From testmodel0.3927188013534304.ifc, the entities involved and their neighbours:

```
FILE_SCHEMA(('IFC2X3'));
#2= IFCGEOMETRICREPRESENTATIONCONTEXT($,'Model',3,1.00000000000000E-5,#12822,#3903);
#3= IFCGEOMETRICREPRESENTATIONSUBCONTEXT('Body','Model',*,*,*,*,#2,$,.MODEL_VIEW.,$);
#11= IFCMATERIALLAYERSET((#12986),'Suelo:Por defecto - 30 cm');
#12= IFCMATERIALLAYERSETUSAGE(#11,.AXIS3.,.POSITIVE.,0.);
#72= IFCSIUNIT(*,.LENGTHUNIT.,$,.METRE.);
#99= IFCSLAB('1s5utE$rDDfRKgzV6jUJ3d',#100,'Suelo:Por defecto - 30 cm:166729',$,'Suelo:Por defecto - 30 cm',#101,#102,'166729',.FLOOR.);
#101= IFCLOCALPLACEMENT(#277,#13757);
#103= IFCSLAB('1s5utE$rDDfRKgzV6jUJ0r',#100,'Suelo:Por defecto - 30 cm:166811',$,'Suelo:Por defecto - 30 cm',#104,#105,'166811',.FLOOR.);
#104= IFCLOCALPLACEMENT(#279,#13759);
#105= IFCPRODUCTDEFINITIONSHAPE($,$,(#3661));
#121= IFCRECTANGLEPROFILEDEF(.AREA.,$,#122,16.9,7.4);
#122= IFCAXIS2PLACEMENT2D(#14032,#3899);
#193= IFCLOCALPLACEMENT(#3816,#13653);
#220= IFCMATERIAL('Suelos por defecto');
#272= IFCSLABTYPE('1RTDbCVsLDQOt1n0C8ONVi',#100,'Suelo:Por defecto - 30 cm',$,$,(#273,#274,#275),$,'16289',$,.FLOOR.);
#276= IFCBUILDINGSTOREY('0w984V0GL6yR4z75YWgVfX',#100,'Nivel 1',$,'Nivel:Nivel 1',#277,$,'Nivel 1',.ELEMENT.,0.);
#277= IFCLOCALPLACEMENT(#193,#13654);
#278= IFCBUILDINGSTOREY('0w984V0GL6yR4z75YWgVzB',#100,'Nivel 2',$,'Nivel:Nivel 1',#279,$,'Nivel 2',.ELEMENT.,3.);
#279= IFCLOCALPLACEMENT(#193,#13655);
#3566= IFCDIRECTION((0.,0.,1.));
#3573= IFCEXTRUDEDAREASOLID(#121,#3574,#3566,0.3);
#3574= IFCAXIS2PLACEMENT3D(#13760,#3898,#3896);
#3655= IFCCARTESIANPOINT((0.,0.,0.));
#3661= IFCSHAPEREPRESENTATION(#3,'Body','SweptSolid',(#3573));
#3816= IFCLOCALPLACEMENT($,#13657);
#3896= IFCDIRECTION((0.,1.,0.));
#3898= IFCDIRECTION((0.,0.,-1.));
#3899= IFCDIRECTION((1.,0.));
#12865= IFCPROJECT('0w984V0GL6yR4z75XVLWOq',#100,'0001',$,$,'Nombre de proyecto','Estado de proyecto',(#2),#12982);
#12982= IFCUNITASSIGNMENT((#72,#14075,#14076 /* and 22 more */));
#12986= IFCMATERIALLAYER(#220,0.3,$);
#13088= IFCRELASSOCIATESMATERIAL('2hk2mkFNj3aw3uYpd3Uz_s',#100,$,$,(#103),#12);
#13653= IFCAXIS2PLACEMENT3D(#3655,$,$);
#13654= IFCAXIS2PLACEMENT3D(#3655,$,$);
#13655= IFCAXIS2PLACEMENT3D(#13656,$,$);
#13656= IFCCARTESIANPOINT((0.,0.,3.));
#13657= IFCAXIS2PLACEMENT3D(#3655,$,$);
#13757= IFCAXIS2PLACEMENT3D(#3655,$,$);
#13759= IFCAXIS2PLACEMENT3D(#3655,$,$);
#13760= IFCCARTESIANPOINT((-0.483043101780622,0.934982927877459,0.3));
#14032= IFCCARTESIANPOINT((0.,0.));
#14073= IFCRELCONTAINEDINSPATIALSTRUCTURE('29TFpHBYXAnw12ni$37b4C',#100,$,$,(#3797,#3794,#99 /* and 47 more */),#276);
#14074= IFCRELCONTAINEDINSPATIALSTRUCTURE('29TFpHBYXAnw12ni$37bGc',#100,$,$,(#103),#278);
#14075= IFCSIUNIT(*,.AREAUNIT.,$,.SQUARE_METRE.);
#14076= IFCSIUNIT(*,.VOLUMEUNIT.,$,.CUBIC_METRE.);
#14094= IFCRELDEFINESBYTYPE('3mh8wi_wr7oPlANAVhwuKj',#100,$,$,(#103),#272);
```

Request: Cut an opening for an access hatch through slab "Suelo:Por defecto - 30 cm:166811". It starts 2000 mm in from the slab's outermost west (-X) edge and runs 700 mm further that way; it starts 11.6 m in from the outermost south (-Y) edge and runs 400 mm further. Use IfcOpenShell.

```python
import numpy as np
import ifcopenshell
import ifcopenshell.api.feature
import ifcopenshell.api.geometry
import ifcopenshell.api.root
import ifcopenshell.geom
import ifcopenshell.util.placement
import ifcopenshell.util.representation
import ifcopenshell.util.shape
import ifcopenshell.util.unit

model = ifcopenshell.open("testmodel0.3927188013534304.ifc")
unit_scale = ifcopenshell.util.unit.calculate_unit_scale(model)
settings = ifcopenshell.geom.settings()


def volume(element):
    """Net volume in cubic metres, openings subtracted."""
    shape = ifcopenshell.geom.create_shape(settings, element)
    return ifcopenshell.util.shape.get_volume(shape.geometry)


slab = model.by_id(103)
before = volume(slab)

# Extent in the slab's own axes, in metres. The edges named are its -X and -Y sides.
slab_shape = ifcopenshell.geom.create_shape(settings, slab)
vertices = ifcopenshell.util.shape.get_vertices(slab_shape.geometry)
x_min, y_min, bottom = vertices.min(axis=0)
top = vertices[:, 2].max()

opening = ifcopenshell.api.root.create_entity(model, ifc_class="IfcOpeningElement", name="Access hatch opening")
context = ifcopenshell.util.representation.get_context(model, "Model", "Body", "MODEL_VIEW")
width, depth = 0.7, 0.4
outline = [(0.0, 0.0), (width, 0.0), (width, depth), (0.0, depth), (0.0, 0.0)]
# Overshoot both faces by 50 mm so the cut is clean.
shape = ifcopenshell.api.geometry.add_slab_representation(
    model, context=context, depth=top - bottom + 0.1, polyline=outline
)
ifcopenshell.api.geometry.assign_representation(model, product=opening, representation=shape)

matrix = ifcopenshell.util.placement.get_local_placement(slab.ObjectPlacement)
matrix[:, 3] = matrix @ np.append(np.array([x_min + 2, y_min + 11.6, bottom - 0.05]) / unit_scale, 1.0)
ifcopenshell.api.geometry.edit_object_placement(model, product=opening, matrix=matrix, is_si=False)
ifcopenshell.api.feature.add_feature(model, feature=opening, element=slab)

after = volume(slab)

print(f"slab volume {before:.3f} -> {after:.3f} m3")

model.write("testmodel0.3927188013534304_updated.ifc")
```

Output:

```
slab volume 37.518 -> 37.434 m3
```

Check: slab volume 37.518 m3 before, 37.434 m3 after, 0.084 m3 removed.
